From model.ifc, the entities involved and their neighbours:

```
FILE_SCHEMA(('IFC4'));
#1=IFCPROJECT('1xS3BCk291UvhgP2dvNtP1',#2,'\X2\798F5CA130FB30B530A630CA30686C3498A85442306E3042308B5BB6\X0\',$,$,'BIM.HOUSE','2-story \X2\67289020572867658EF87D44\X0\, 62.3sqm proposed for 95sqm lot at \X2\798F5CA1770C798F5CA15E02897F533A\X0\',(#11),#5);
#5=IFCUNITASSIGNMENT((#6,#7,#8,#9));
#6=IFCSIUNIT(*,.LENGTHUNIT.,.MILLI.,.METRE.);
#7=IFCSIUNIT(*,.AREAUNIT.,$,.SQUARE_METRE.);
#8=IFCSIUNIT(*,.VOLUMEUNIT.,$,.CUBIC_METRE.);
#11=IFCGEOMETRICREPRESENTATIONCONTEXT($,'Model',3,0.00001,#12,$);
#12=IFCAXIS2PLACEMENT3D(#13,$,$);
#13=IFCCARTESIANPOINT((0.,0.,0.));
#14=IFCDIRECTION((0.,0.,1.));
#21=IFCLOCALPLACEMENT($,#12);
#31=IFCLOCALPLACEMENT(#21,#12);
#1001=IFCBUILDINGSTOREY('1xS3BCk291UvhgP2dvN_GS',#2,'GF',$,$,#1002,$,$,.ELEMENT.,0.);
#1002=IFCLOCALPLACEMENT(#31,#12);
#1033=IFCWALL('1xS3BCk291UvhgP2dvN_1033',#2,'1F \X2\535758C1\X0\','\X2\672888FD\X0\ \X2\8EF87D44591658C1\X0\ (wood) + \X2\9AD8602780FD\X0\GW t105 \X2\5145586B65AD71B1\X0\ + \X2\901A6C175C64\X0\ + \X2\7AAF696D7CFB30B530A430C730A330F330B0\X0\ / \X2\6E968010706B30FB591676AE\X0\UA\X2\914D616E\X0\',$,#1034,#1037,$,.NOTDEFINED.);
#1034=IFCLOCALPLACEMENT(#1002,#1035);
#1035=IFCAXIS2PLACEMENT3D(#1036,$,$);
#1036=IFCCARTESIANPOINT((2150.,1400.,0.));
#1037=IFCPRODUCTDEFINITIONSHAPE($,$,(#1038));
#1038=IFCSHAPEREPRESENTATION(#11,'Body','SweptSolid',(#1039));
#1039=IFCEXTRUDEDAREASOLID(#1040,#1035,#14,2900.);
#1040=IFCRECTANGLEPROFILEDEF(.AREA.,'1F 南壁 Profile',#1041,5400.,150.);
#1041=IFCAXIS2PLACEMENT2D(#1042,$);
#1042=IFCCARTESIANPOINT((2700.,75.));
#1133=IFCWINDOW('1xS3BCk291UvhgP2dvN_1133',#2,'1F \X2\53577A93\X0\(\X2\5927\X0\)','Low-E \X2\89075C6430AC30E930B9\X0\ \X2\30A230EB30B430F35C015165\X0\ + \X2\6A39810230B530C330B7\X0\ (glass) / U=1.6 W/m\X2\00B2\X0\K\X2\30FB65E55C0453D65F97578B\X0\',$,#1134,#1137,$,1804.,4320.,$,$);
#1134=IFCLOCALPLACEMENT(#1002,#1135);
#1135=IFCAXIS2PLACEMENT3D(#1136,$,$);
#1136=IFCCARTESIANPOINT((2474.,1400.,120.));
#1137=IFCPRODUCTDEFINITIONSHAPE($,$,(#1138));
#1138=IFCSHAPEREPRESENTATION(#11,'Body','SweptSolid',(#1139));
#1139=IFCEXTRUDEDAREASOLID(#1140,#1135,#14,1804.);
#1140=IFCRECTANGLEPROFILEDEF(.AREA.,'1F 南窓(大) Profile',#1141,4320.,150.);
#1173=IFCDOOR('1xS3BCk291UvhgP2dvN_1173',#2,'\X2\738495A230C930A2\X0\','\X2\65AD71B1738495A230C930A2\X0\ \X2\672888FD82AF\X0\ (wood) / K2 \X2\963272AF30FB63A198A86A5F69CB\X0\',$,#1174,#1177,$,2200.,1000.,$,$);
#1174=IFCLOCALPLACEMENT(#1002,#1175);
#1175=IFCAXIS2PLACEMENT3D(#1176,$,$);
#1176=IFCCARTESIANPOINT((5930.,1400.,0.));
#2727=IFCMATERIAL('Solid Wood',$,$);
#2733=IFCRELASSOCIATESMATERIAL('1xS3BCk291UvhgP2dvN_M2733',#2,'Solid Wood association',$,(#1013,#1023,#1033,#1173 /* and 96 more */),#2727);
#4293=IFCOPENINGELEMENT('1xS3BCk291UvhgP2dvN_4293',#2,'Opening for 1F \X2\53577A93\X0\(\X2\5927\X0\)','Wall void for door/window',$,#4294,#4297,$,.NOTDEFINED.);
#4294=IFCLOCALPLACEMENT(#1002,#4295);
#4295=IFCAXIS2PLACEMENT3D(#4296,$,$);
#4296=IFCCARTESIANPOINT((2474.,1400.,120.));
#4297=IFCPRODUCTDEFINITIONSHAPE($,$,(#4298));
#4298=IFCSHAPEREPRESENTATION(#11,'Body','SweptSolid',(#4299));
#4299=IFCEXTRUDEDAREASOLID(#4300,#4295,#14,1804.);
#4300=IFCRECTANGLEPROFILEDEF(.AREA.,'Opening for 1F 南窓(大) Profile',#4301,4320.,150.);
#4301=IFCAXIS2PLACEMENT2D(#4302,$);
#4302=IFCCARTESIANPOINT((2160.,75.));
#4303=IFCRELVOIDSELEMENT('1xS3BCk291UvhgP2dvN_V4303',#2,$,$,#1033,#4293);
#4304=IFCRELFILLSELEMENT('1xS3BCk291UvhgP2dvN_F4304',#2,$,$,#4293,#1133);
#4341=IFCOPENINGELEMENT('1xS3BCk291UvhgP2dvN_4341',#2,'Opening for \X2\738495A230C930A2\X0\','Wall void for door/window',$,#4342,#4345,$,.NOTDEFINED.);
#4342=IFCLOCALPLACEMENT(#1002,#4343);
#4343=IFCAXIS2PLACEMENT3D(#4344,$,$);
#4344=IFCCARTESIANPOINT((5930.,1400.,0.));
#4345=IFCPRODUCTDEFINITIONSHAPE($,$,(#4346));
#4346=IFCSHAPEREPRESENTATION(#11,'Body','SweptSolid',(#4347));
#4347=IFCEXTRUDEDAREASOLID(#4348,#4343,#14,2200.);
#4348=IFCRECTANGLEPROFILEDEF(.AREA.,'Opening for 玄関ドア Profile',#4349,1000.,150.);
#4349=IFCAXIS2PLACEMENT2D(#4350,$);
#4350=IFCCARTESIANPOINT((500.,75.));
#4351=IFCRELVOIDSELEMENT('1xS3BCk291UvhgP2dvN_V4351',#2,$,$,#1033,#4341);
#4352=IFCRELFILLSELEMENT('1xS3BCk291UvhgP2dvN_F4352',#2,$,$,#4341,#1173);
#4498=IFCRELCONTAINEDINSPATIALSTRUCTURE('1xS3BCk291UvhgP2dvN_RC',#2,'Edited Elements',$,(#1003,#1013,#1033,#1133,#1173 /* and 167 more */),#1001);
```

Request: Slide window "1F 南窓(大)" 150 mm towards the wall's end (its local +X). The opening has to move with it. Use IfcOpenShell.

```python
import ifcopenshell
import ifcopenshell.api.geometry
import ifcopenshell.util.placement
import ifcopenshell.util.unit

model = ifcopenshell.open("model.ifc")
unit_scale = ifcopenshell.util.unit.calculate_unit_scale(model)

window = model.by_guid("1xS3BCk291UvhgP2dvN_1133")
opening = window.FillsVoids[0].RelatingOpeningElement
wall = opening.VoidsElements[0].RelatingBuildingElement

wall_matrix = ifcopenshell.util.placement.get_local_placement(wall.ObjectPlacement)
shift = wall_matrix[:3, 0] * 0.15 / unit_scale
before = ifcopenshell.util.placement.get_local_placement(window.ObjectPlacement)[:3, 3].copy()

# The window is not placed relative to its opening, so move both.
for product in (opening, window):
    matrix = ifcopenshell.util.placement.get_local_placement(product.ObjectPlacement)
    matrix[:3, 3] += shift
    ifcopenshell.api.geometry.edit_object_placement(model, product=product, matrix=matrix, is_si=False)

after = ifcopenshell.util.placement.get_local_placement(window.ObjectPlacement)[:3, 3]
print("window moved by", (after - before).round(3) + 0.0)

model.write("model-out.ifc")
```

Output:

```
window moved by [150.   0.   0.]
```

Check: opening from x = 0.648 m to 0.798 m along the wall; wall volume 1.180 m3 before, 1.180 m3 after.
